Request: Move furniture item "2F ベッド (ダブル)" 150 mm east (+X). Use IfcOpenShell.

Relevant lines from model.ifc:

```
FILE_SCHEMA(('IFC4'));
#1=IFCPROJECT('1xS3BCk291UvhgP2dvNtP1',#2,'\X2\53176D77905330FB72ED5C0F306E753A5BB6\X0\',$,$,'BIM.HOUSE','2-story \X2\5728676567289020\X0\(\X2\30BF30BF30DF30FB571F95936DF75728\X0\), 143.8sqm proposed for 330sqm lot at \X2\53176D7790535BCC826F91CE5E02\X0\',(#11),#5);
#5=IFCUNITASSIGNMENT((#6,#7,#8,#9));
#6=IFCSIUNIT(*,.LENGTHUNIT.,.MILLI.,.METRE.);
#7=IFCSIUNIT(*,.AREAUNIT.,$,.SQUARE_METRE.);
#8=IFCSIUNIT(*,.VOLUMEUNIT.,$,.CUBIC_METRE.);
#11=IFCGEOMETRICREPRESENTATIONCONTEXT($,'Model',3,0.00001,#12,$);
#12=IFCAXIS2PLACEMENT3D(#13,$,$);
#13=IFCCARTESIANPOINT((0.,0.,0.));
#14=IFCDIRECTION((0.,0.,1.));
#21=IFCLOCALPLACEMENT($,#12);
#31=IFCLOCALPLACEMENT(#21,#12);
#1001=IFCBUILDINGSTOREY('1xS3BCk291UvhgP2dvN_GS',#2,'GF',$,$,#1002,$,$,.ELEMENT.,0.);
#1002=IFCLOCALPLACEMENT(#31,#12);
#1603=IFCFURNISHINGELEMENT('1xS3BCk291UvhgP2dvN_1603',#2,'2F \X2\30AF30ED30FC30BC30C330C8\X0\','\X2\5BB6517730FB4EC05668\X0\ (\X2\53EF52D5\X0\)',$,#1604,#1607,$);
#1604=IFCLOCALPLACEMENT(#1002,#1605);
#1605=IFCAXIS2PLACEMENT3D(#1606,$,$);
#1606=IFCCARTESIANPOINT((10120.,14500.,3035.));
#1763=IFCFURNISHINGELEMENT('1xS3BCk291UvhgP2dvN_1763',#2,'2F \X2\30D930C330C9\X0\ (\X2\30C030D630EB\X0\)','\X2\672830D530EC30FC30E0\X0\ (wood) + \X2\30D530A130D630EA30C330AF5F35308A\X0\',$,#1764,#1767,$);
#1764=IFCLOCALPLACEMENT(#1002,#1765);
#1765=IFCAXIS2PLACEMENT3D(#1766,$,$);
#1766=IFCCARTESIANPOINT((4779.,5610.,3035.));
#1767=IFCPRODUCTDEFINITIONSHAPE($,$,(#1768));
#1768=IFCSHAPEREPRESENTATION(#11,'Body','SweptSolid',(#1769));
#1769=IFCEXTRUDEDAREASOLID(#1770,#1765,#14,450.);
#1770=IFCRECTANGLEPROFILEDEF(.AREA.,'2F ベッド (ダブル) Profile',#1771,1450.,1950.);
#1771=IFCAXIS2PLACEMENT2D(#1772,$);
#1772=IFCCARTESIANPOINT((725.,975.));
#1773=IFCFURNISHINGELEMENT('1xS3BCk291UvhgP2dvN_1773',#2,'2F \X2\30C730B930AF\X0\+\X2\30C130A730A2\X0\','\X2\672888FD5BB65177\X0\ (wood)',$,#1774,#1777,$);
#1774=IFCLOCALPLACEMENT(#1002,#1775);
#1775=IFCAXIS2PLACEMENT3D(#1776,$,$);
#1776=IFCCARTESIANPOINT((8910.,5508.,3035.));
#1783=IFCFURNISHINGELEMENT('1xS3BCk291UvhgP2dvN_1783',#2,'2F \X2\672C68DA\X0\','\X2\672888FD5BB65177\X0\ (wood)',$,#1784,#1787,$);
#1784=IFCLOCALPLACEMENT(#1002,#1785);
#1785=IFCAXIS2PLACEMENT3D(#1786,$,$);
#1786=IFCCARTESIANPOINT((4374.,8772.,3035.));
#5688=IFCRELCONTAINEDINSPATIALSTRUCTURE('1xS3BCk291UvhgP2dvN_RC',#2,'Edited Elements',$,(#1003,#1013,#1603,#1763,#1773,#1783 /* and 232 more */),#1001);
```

```python
import ifcopenshell
import ifcopenshell.api.geometry
import ifcopenshell.util.placement

model = ifcopenshell.open("model.ifc")

item = model.by_guid("1xS3BCk291UvhgP2dvN_1763")
matrix = ifcopenshell.util.placement.get_local_placement(item.ObjectPlacement)
matrix[0, 3] += 150.0
ifcopenshell.api.geometry.edit_object_placement(model, product=item, matrix=matrix, is_si=False)

print(ifcopenshell.util.placement.get_local_placement(item.ObjectPlacement).round(3) + 0.0)

model.write("model_edited.ifc")
```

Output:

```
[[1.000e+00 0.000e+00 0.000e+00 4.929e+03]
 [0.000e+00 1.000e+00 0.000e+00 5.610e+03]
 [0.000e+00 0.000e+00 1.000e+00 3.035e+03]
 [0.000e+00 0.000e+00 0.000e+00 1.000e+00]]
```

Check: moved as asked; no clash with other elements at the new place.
